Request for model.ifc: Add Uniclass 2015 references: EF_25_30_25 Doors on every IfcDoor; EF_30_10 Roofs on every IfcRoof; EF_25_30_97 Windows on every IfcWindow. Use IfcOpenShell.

First a look at what the model holds.

```python
import ifcopenshell

model = ifcopenshell.open("model.ifc")
print(model.schema)
print("classifications:", [c.Name for c in model.by_type("IfcClassification")])
for ifc_class in ("IfcDoor", "IfcRoof", "IfcStair", "IfcWall", "IfcWindow"):
    print(ifc_class, len(model.by_type(ifc_class)))
```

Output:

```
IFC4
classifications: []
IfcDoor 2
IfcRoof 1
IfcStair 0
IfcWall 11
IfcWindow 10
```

```python
import ifcopenshell
import ifcopenshell.api.classification

model = ifcopenshell.open("model.ifc")

system = ifcopenshell.api.classification.add_classification(model, classification="Uniclass 2015")

codes = {
    "IfcDoor": ("EF_25_30_25", "Doors"),
    "IfcRoof": ("EF_30_10", "Roofs"),
    "IfcWindow": ("EF_25_30_97", "Windows"),
}
for ifc_class, (code, name) in codes.items():
    products = model.by_type(ifc_class)
    ifcopenshell.api.classification.add_reference(
        model, products=products, classification=system, identification=code, name=name
    )
    print(code, len(products))

model.write("model_rev.ifc")
```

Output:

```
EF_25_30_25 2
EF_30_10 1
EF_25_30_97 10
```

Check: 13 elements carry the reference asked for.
